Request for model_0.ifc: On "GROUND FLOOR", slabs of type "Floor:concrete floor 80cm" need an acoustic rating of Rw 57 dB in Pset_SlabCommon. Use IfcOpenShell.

First a look at what the model holds.

```python
import ifcopenshell
import ifcopenshell.util.element

model = ifcopenshell.open("model_0.ifc")
print(model.schema)
storey = next(s for s in model.by_type("IfcBuildingStorey") if s.Name == "GROUND FLOOR")
slabs = [e for e in ifcopenshell.util.element.get_decomposition(storey) if e.is_a("IfcSlab")]
seen = {}
for e in slabs:
    element_type = ifcopenshell.util.element.get_type(e)
    key = (element_type.Name if element_type != e and element_type else None, ifcopenshell.util.element.get_pset(e, "Pset_SlabCommon", "AcousticRating"))
    seen[key] = seen.get(key, 0) + 1
for (name, value), count in sorted(seen.items(), key=str):
    print(count, "x", name, "|", value)
```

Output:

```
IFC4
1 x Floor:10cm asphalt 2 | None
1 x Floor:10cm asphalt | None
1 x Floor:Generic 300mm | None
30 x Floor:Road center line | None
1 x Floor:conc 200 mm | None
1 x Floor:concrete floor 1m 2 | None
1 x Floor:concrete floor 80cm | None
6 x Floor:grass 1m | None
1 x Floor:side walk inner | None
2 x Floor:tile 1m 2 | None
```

```python
import ifcopenshell
import ifcopenshell.api.pset
import ifcopenshell.util.element

model = ifcopenshell.open("model_0.ifc")

storey = next(s for s in model.by_type("IfcBuildingStorey") if s.Name == "GROUND FLOOR")
slabs = [e for e in ifcopenshell.util.element.get_decomposition(storey) if e.is_a("IfcSlab")]

count = 0
for e in slabs:
    element_type = ifcopenshell.util.element.get_type(e)
    if element_type in (None, e) or element_type.Name != "Floor:concrete floor 80cm":
        continue
    # add_pset returns the element's existing set when there is one.
    pset = ifcopenshell.api.pset.add_pset(model, product=e, name="Pset_SlabCommon")
    ifcopenshell.api.pset.edit_pset(model, pset=pset, properties={"AcousticRating": "Rw 57 dB"})
    count += 1

print(count, "slabs updated")

model.write("model_0-out.ifc")
```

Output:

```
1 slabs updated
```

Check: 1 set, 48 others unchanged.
